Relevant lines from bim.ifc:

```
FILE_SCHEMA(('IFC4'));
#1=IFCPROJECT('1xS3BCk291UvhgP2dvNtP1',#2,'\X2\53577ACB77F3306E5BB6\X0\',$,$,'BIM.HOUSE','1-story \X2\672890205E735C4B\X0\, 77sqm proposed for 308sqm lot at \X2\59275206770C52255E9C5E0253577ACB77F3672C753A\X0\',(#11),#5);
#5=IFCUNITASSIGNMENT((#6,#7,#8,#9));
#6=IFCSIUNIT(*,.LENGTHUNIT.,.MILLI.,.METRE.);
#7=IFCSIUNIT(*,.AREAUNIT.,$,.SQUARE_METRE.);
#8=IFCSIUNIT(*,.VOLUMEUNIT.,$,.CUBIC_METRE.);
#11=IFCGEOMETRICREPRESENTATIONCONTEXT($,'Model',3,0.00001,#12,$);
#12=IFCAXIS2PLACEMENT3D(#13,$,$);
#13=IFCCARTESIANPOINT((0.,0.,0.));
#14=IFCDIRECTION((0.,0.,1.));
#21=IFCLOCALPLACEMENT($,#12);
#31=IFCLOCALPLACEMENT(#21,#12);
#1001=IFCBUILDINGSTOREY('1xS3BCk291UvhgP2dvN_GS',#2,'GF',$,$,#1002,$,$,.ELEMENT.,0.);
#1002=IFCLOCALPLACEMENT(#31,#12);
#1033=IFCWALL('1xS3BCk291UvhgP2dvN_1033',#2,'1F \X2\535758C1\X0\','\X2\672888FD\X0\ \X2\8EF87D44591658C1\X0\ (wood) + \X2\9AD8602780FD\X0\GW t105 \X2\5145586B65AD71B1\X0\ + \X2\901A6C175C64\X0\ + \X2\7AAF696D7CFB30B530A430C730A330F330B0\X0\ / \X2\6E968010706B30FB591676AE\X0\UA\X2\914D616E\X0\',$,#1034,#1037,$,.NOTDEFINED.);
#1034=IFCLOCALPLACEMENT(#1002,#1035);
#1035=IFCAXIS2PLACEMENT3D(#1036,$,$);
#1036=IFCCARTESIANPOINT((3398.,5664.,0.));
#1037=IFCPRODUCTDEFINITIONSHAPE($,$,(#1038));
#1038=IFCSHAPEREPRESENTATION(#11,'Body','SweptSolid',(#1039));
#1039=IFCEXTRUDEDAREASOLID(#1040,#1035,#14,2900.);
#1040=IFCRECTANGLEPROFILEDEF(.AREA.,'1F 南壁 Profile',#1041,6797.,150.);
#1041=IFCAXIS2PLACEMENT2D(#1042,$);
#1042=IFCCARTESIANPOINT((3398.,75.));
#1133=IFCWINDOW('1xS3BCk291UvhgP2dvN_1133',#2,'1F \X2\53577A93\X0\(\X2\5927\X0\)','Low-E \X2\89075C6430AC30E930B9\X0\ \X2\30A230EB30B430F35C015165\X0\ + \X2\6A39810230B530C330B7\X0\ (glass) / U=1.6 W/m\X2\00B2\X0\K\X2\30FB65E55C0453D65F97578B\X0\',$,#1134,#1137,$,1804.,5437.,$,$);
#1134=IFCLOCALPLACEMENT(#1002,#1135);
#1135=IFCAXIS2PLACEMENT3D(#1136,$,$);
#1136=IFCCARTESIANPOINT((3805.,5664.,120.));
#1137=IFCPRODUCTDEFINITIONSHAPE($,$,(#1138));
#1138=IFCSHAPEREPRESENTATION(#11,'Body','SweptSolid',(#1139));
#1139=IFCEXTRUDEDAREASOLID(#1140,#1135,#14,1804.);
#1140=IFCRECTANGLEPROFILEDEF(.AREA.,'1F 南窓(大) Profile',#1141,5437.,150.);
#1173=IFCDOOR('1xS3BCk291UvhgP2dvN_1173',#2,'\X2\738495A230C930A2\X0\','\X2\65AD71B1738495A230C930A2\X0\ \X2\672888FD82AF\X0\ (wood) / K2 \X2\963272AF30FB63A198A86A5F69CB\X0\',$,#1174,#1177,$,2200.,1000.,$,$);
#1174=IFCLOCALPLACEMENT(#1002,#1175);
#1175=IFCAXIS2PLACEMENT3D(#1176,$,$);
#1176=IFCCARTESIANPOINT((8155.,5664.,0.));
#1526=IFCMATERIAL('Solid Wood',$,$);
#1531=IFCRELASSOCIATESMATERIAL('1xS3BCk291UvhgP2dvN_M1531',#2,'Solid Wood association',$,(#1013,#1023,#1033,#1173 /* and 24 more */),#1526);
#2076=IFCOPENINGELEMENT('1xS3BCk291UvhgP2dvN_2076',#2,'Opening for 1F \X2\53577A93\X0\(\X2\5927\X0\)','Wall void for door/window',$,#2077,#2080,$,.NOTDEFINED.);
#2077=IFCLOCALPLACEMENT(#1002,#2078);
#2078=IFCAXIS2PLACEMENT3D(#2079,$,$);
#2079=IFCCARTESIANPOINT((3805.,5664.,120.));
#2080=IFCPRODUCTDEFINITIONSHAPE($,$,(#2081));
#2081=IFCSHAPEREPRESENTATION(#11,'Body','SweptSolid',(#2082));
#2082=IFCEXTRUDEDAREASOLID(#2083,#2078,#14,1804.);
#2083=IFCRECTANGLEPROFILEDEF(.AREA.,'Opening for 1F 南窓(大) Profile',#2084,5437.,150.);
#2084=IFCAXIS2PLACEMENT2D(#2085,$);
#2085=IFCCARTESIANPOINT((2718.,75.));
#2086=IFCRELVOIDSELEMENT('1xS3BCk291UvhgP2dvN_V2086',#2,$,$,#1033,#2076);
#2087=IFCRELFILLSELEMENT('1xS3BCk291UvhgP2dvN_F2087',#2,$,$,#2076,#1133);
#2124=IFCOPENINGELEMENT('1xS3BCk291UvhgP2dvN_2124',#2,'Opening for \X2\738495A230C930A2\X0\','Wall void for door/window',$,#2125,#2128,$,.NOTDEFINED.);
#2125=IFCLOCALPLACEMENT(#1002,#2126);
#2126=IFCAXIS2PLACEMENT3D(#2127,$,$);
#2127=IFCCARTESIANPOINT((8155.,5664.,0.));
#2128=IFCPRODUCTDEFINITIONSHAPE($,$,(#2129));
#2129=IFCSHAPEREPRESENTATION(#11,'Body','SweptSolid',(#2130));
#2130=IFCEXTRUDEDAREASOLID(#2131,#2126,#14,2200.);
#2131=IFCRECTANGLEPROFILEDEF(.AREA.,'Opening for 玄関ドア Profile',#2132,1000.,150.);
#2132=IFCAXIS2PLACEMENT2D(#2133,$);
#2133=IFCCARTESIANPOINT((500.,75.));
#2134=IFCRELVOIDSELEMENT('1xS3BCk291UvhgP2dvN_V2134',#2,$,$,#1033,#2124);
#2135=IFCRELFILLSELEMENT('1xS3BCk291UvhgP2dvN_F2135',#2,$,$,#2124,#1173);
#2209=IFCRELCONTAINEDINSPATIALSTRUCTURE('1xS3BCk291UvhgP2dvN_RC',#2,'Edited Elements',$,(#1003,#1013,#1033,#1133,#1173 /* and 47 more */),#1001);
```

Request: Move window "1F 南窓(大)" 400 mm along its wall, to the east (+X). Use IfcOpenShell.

```python
import ifcopenshell
import ifcopenshell.api.geometry
import ifcopenshell.util.placement
import ifcopenshell.util.unit

model = ifcopenshell.open("bim.ifc")
unit_scale = ifcopenshell.util.unit.calculate_unit_scale(model)

window = model.by_id(1133)
opening = window.FillsVoids[0].RelatingOpeningElement
wall = opening.VoidsElements[0].RelatingBuildingElement

wall_matrix = ifcopenshell.util.placement.get_local_placement(wall.ObjectPlacement)
shift = wall_matrix[:3, 0] * 0.4 / unit_scale
before = ifcopenshell.util.placement.get_local_placement(window.ObjectPlacement)[:3, 3].copy()

# The window is not placed relative to its opening, so move both.
for product in (opening, window):
    matrix = ifcopenshell.util.placement.get_local_placement(product.ObjectPlacement)
    matrix[:3, 3] += shift
    ifcopenshell.api.geometry.edit_object_placement(model, product=product, matrix=matrix, is_si=False)

after = ifcopenshell.util.placement.get_local_placement(window.ObjectPlacement)[:3, 3]
print("window moved by", (after - before).round(3) + 0.0)

model.write("bim_rev.ifc")
```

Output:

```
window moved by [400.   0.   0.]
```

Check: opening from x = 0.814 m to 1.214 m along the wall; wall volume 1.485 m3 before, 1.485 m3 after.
